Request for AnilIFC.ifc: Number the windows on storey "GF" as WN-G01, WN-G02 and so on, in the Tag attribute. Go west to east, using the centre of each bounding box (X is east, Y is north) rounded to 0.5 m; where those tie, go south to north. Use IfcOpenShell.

First a look at what the model holds.

```python
import ifcopenshell
import ifcopenshell.util.element
import ifcopenshell.util.placement

model = ifcopenshell.open("AnilIFC.ifc")
print(model.schema)
storey = next(s for s in model.by_type("IfcBuildingStorey") if s.Name == "GF")
windows = [e for e in ifcopenshell.util.element.get_decomposition(storey) if e.is_a("IfcWindow")]
for e in sorted(windows, key=lambda e: e.id()):
    origin = ifcopenshell.util.placement.get_local_placement(e.ObjectPlacement)[:3, 3]
    print(e.id(), e.Tag, e.Name, origin.round(2) + 0.0, sep=" | ")
```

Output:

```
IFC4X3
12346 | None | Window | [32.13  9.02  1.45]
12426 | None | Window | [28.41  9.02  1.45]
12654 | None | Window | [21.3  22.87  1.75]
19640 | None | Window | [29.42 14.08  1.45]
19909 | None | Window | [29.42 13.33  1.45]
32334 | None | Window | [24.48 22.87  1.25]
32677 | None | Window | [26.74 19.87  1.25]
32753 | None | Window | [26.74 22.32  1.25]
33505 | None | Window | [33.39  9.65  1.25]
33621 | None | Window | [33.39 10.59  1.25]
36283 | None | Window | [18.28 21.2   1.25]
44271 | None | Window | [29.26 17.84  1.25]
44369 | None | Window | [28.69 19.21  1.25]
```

```python
import ifcopenshell
import ifcopenshell.geom
import ifcopenshell.util.element
import ifcopenshell.util.shape

model = ifcopenshell.open("AnilIFC.ifc")
settings = ifcopenshell.geom.settings()
settings.set("use-world-coords", True)


def centre(element):
    shape = ifcopenshell.geom.create_shape(settings, element)
    return ifcopenshell.util.shape.get_bbox_centroid(shape.geometry)


storey = next(s for s in model.by_type("IfcBuildingStorey") if s.Name == "GF")
windows = [e for e in ifcopenshell.util.element.get_decomposition(storey) if e.is_a("IfcWindow")]

# Insertion points can sit at a corner or the storey origin, so sort by the geometry (in metres).
centres = {e: centre(e) for e in windows}
windows.sort(key=lambda e: (round(centres[e][0] / 0.5), centres[e][1]))

for i, e in enumerate(windows, start=1):
    number = f"WN-G{i:02d}"
    e.Tag = number
    print(e.id(), number)

model.write("AnilIFC_updated.ifc")
```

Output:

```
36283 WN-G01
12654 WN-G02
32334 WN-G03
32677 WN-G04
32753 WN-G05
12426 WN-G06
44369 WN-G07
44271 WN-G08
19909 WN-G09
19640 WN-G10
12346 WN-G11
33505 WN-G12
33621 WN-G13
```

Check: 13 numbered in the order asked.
